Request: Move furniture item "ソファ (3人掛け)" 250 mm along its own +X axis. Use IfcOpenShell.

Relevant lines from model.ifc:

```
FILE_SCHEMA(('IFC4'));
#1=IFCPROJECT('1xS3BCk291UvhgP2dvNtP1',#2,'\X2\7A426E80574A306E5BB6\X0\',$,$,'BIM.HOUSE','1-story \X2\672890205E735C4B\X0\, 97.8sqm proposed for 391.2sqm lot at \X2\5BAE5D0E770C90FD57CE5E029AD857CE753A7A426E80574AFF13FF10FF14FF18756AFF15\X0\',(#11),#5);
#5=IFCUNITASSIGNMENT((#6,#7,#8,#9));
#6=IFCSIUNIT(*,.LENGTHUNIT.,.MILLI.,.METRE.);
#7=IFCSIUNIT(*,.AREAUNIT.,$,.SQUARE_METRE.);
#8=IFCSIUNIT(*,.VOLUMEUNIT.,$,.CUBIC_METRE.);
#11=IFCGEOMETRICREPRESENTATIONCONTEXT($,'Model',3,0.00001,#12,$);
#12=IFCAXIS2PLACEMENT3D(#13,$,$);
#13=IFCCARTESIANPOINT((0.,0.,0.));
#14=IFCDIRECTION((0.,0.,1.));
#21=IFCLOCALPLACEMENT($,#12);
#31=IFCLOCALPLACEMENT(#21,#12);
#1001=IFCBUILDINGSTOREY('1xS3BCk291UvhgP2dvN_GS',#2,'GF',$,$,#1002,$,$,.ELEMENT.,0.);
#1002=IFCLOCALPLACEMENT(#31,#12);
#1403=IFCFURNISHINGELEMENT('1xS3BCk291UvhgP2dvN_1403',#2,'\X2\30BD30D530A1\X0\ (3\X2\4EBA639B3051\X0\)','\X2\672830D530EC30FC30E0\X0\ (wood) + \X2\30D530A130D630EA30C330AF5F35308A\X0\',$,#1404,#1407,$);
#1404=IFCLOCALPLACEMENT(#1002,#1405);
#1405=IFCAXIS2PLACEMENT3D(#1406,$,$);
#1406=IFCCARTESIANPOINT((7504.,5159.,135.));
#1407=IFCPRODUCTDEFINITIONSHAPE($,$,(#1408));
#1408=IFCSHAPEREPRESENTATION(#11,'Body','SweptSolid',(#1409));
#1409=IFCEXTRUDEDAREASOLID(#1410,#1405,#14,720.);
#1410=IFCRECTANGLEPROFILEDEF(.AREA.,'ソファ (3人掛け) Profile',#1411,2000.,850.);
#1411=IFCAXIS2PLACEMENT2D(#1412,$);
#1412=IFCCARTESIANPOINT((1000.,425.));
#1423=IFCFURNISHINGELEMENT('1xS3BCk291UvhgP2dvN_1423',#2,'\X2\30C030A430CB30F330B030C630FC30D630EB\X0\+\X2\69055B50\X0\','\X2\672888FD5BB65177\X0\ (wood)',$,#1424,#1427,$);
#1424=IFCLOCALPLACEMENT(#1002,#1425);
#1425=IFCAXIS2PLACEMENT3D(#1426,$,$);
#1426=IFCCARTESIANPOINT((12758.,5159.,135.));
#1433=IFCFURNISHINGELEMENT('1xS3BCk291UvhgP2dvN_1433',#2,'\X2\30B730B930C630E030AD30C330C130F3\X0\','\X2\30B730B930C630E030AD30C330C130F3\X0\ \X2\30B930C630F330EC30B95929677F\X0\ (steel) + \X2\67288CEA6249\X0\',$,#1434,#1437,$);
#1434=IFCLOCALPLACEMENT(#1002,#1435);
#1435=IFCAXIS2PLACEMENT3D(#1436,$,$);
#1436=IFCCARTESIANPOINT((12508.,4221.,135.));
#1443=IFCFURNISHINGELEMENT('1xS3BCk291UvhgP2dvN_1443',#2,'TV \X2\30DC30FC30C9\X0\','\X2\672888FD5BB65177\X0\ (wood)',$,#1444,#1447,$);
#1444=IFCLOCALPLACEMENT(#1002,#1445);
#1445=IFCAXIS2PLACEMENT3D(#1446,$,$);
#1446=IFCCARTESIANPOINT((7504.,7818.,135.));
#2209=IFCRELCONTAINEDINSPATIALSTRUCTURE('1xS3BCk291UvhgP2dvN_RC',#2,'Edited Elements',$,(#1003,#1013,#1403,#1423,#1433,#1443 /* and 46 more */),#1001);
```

```python
import ifcopenshell
import ifcopenshell.api.geometry
import ifcopenshell.util.placement

model = ifcopenshell.open("model.ifc")

item = model.by_guid("1xS3BCk291UvhgP2dvN_1403")
matrix = ifcopenshell.util.placement.get_local_placement(item.ObjectPlacement)
matrix[:3, 3] += matrix[:3, 0] * 250.0
ifcopenshell.api.geometry.edit_object_placement(model, product=item, matrix=matrix, is_si=False)

print(ifcopenshell.util.placement.get_local_placement(item.ObjectPlacement).round(3) + 0.0)

model.write("model_edited.ifc")
```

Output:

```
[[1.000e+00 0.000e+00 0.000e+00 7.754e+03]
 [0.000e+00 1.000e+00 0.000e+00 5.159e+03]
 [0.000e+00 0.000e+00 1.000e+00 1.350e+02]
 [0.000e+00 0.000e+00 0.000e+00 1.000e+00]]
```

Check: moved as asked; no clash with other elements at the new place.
